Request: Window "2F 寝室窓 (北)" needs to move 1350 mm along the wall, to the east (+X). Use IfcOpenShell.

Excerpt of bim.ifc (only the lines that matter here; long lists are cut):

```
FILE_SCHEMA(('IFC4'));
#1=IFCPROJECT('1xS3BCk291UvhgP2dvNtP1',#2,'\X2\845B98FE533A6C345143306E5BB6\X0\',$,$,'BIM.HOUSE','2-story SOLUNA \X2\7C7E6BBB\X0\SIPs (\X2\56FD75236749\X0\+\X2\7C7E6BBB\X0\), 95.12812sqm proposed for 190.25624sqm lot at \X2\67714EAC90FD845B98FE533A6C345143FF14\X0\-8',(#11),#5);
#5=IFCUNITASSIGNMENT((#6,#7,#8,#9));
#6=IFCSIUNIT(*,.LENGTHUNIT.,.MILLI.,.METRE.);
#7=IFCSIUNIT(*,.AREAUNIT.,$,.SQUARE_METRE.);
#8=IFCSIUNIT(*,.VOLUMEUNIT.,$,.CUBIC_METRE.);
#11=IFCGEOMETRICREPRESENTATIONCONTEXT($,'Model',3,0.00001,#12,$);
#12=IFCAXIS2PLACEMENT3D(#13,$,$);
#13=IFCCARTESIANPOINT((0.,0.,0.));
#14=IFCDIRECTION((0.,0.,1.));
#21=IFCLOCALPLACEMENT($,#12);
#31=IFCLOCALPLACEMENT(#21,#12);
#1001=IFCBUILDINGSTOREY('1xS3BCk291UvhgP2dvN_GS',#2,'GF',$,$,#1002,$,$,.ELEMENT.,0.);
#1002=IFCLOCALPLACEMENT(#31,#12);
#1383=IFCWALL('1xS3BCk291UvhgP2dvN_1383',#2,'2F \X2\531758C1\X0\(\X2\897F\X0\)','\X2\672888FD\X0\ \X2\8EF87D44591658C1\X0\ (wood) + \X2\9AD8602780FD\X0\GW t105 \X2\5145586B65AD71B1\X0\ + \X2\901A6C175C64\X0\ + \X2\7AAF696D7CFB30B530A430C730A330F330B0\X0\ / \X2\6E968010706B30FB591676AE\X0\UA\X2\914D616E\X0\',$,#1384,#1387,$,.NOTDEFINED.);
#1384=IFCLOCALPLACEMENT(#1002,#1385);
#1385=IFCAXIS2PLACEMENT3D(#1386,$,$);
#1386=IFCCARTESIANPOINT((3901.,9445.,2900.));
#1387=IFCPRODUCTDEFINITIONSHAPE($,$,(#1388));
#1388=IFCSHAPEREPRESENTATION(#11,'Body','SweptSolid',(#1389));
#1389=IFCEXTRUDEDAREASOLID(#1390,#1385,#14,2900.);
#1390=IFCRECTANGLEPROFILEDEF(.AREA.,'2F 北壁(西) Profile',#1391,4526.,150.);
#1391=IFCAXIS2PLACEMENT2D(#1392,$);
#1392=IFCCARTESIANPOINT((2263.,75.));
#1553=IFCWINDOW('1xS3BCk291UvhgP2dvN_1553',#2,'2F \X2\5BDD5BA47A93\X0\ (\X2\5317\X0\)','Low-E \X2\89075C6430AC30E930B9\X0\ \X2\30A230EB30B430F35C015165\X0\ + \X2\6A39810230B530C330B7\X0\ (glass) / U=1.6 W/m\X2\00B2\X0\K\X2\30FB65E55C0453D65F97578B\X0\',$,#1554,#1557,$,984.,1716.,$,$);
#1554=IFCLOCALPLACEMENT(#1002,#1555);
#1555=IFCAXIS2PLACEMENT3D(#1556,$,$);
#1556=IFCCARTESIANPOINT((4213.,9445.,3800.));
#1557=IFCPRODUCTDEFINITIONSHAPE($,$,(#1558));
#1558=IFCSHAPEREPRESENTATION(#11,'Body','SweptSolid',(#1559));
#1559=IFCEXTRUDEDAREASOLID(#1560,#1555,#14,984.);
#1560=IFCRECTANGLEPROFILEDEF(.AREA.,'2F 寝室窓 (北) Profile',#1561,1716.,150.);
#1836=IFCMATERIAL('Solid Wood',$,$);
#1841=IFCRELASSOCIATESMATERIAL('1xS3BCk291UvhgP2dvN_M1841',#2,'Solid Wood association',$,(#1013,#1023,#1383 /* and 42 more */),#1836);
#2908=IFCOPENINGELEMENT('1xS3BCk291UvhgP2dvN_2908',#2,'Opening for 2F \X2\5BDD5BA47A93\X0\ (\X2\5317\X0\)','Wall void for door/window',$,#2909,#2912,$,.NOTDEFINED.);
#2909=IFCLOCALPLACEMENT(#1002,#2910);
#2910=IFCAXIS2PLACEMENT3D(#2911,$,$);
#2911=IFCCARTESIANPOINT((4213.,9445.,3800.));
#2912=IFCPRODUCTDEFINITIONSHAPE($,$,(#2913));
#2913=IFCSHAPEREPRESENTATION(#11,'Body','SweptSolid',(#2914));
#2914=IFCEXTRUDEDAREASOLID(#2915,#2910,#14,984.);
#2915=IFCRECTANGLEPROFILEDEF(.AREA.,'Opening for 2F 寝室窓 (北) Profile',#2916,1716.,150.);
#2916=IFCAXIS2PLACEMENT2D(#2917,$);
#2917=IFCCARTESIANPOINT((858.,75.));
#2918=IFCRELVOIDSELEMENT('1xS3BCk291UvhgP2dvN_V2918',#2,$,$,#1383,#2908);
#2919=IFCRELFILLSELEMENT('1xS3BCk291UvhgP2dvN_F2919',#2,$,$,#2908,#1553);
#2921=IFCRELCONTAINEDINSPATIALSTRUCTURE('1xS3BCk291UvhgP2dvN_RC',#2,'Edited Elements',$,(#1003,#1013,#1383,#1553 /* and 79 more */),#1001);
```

```python
import ifcopenshell
import ifcopenshell.api.geometry
import ifcopenshell.util.placement
import ifcopenshell.util.unit

model = ifcopenshell.open("bim.ifc")
unit_scale = ifcopenshell.util.unit.calculate_unit_scale(model)

window = model.by_guid("1xS3BCk291UvhgP2dvN_1553")
opening = window.FillsVoids[0].RelatingOpeningElement
wall = opening.VoidsElements[0].RelatingBuildingElement

wall_matrix = ifcopenshell.util.placement.get_local_placement(wall.ObjectPlacement)
shift = wall_matrix[:3, 0] * 1.35 / unit_scale
before = ifcopenshell.util.placement.get_local_placement(window.ObjectPlacement)[:3, 3].copy()

# The window is not placed relative to its opening, so move both.
for product in (opening, window):
    matrix = ifcopenshell.util.placement.get_local_placement(product.ObjectPlacement)
    matrix[:3, 3] += shift
    ifcopenshell.api.geometry.edit_object_placement(model, product=product, matrix=matrix, is_si=False)

after = ifcopenshell.util.placement.get_local_placement(window.ObjectPlacement)[:3, 3]
print("window moved by", (after - before).round(3) + 0.0)

model.write("bim_rev.ifc")
```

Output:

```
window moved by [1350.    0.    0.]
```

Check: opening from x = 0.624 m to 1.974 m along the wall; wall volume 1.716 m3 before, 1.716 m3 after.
